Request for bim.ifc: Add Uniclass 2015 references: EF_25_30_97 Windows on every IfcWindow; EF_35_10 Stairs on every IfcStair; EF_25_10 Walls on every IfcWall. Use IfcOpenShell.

First a look at what the model holds.

```python
import ifcopenshell

model = ifcopenshell.open("bim.ifc")
print(model.schema)
print("classifications:", [c.Name for c in model.by_type("IfcClassification")])
for ifc_class in ("IfcDoor", "IfcRoof", "IfcStair", "IfcWall", "IfcWindow"):
    print(ifc_class, len(model.by_type(ifc_class)))
```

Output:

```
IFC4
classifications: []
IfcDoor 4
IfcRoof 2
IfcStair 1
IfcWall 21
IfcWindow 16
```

```python
import ifcopenshell
import ifcopenshell.api.classification

model = ifcopenshell.open("bim.ifc")

system = ifcopenshell.api.classification.add_classification(model, classification="Uniclass 2015")

codes = {
    "IfcWindow": ("EF_25_30_97", "Windows"),
    "IfcStair": ("EF_35_10", "Stairs"),
    "IfcWall": ("EF_25_10", "Walls"),
}
for ifc_class, (code, name) in codes.items():
    products = model.by_type(ifc_class)
    ifcopenshell.api.classification.add_reference(
        model, products=products, classification=system, identification=code, name=name
    )
    print(code, len(products))

model.write("bim_v2.ifc")
```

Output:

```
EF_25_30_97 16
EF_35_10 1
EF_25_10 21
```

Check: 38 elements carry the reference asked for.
